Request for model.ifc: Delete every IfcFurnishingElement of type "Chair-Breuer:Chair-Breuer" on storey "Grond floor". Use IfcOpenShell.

First a look at what the model holds.

```python
import ifcopenshell
import ifcopenshell.util.element

model = ifcopenshell.open("model.ifc")
print(model.schema)
storey = next(s for s in model.by_type("IfcBuildingStorey") if s.Name == "Grond floor")
furniture = [e for e in ifcopenshell.util.element.get_decomposition(storey) if e.is_a("IfcFurnishingElement")]
seen = {}
for e in furniture:
    element_type = ifcopenshell.util.element.get_type(e)
    name = element_type.Name if element_type not in (None, e) else None
    seen[name] = seen.get(name, 0) + 1
for name, count in sorted(seen.items(), key=str):
    print(count, "x", name)
```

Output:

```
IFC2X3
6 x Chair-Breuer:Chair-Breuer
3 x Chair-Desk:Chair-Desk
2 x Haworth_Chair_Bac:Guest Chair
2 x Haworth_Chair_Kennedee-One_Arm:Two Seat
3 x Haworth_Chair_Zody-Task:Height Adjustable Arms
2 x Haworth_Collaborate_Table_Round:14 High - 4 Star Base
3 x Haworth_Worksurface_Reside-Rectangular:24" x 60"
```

```python
import ifcopenshell
import ifcopenshell.api.root
import ifcopenshell.util.element

model = ifcopenshell.open("model.ifc")

storey = next(s for s in model.by_type("IfcBuildingStorey") if s.Name == "Grond floor")
furniture = [e for e in ifcopenshell.util.element.get_decomposition(storey) if e.is_a("IfcFurnishingElement")]
targets = [e for e in furniture if (t := ifcopenshell.util.element.get_type(e)) not in (None, e) and t.Name == "Chair-Breuer:Chair-Breuer"]

for e in targets:
    ifcopenshell.api.root.remove_product(model, product=e)
print(len(targets), "removed")

model.write("model_v2.ifc")
```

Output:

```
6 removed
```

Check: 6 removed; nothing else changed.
